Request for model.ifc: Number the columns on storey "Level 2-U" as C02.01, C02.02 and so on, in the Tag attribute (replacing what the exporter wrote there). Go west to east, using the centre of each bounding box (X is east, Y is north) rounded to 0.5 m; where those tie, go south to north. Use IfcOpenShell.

First a look at what the model holds.

```python
import ifcopenshell
import ifcopenshell.util.element
import ifcopenshell.util.placement

model = ifcopenshell.open("model.ifc")
print(model.schema)
storey = next(s for s in model.by_type("IfcBuildingStorey") if s.Name == "Level 2-U")
columns = [e for e in ifcopenshell.util.element.get_decomposition(storey) if e.is_a("IfcColumn")]
for e in sorted(columns, key=lambda e: e.id()):
    origin = ifcopenshell.util.placement.get_local_placement(e.ObjectPlacement)[:3, 3]
    print(e.id(), e.Tag, e.Name, origin.round(2) + 0.0, sep=" | ")
```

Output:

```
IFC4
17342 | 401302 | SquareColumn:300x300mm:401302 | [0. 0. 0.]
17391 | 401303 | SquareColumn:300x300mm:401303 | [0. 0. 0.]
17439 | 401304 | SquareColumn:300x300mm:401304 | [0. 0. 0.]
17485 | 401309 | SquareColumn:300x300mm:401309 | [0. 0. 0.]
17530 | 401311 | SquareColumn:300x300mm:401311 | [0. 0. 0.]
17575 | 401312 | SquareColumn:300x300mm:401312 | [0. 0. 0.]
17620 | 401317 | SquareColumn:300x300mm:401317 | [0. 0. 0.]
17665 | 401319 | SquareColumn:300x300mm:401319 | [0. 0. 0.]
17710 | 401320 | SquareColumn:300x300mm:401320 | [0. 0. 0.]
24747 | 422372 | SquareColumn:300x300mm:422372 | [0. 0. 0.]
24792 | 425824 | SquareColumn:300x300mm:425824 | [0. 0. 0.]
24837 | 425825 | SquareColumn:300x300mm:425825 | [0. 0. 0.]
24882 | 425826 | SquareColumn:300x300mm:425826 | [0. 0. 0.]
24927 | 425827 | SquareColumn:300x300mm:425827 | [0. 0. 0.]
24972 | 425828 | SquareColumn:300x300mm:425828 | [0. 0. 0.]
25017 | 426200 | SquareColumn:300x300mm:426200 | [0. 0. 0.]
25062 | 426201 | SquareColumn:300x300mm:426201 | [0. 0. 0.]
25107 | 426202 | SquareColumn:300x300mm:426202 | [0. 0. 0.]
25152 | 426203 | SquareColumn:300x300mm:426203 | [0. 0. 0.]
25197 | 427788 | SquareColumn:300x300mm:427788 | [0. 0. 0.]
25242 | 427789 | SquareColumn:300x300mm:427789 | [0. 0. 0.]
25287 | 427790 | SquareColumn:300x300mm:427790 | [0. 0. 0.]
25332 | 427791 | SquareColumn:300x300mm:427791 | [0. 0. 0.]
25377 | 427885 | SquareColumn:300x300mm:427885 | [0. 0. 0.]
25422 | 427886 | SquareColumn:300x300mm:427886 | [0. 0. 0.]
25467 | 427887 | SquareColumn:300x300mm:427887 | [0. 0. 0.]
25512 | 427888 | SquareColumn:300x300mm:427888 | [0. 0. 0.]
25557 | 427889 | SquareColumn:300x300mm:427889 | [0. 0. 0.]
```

```python
import ifcopenshell
import ifcopenshell.geom
import ifcopenshell.util.element
import ifcopenshell.util.shape

model = ifcopenshell.open("model.ifc")
settings = ifcopenshell.geom.settings()
settings.set("use-world-coords", True)


def centre(element):
    shape = ifcopenshell.geom.create_shape(settings, element)
    return ifcopenshell.util.shape.get_bbox_centroid(shape.geometry)


storey = next(s for s in model.by_type("IfcBuildingStorey") if s.Name == "Level 2-U")
columns = [e for e in ifcopenshell.util.element.get_decomposition(storey) if e.is_a("IfcColumn")]

# Insertion points can sit at a corner or the storey origin, so sort by the geometry (in metres).
centres = {e: centre(e) for e in columns}
columns.sort(key=lambda e: (round(centres[e][0] / 0.5), centres[e][1]))

for i, e in enumerate(columns, start=1):
    number = f"C02.{i:02d}"
    e.Tag = number
    print(e.id(), number)

model.write("model_edited.ifc")
```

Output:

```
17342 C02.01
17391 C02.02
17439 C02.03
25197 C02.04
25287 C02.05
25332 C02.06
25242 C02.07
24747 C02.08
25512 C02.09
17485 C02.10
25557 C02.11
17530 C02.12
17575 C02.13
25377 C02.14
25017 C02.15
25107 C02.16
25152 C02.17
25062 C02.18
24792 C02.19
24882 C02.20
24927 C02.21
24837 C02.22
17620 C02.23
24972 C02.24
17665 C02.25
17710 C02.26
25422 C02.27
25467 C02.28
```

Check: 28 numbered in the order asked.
